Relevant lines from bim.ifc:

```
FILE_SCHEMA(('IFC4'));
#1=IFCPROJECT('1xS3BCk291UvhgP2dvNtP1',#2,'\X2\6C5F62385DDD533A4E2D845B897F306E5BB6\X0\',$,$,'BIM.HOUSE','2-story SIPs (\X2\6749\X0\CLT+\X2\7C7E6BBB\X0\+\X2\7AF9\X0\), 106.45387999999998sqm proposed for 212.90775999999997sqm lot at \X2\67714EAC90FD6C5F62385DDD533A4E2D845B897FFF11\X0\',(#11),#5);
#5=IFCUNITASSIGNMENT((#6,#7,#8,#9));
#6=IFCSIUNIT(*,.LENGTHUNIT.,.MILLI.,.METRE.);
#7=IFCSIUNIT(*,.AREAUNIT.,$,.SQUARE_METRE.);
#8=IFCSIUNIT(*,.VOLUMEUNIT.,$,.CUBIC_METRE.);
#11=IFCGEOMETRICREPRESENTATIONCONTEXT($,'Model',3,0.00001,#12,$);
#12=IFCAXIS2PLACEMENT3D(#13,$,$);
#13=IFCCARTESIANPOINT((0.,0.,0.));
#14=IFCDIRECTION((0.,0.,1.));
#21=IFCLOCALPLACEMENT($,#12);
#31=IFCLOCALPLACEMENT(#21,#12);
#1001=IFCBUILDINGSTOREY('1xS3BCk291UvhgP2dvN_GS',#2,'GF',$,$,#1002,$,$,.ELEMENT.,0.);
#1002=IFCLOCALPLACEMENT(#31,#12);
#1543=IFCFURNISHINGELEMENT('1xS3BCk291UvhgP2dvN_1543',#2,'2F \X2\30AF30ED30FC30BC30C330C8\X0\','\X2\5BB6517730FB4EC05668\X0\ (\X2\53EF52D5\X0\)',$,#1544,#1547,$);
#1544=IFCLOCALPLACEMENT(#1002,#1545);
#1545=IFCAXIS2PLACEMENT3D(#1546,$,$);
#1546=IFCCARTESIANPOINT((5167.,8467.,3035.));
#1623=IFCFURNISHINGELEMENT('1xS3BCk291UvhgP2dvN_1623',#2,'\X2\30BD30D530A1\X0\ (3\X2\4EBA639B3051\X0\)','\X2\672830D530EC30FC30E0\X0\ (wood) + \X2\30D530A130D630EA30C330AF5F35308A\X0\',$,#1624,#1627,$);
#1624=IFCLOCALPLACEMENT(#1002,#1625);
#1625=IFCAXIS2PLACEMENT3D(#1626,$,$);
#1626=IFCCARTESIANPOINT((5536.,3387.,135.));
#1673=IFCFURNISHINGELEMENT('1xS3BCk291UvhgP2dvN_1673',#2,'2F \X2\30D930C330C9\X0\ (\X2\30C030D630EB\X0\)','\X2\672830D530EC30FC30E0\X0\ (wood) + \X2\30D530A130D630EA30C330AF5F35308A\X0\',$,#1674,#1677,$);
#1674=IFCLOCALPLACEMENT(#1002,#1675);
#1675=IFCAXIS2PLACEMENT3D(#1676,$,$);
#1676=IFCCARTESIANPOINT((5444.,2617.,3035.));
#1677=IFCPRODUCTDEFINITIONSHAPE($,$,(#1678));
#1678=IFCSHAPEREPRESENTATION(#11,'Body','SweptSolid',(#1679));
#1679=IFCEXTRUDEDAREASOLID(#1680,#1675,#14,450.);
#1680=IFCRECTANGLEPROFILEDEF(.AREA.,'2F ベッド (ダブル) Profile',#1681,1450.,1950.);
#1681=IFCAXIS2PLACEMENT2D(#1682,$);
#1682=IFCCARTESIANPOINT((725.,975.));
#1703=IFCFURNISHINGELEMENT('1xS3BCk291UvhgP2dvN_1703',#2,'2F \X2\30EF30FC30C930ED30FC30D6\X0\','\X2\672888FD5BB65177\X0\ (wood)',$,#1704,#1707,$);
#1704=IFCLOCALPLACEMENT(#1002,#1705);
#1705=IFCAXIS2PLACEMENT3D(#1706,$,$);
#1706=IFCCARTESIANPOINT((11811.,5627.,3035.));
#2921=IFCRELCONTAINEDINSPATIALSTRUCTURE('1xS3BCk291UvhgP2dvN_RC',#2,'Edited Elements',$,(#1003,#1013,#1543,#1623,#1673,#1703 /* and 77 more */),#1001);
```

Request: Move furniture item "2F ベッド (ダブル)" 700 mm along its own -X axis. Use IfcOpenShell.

```python
import ifcopenshell
import ifcopenshell.api.geometry
import ifcopenshell.util.placement

model = ifcopenshell.open("bim.ifc")

item = model.by_guid("1xS3BCk291UvhgP2dvN_1673")
matrix = ifcopenshell.util.placement.get_local_placement(item.ObjectPlacement)
matrix[:3, 3] -= matrix[:3, 0] * 700.0
ifcopenshell.api.geometry.edit_object_placement(model, product=item, matrix=matrix, is_si=False)

print(ifcopenshell.util.placement.get_local_placement(item.ObjectPlacement).round(3) + 0.0)

model.write("bim-out.ifc")
```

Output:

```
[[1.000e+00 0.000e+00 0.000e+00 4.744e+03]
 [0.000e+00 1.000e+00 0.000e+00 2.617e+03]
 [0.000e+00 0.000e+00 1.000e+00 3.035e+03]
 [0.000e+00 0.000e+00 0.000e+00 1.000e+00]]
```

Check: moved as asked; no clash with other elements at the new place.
